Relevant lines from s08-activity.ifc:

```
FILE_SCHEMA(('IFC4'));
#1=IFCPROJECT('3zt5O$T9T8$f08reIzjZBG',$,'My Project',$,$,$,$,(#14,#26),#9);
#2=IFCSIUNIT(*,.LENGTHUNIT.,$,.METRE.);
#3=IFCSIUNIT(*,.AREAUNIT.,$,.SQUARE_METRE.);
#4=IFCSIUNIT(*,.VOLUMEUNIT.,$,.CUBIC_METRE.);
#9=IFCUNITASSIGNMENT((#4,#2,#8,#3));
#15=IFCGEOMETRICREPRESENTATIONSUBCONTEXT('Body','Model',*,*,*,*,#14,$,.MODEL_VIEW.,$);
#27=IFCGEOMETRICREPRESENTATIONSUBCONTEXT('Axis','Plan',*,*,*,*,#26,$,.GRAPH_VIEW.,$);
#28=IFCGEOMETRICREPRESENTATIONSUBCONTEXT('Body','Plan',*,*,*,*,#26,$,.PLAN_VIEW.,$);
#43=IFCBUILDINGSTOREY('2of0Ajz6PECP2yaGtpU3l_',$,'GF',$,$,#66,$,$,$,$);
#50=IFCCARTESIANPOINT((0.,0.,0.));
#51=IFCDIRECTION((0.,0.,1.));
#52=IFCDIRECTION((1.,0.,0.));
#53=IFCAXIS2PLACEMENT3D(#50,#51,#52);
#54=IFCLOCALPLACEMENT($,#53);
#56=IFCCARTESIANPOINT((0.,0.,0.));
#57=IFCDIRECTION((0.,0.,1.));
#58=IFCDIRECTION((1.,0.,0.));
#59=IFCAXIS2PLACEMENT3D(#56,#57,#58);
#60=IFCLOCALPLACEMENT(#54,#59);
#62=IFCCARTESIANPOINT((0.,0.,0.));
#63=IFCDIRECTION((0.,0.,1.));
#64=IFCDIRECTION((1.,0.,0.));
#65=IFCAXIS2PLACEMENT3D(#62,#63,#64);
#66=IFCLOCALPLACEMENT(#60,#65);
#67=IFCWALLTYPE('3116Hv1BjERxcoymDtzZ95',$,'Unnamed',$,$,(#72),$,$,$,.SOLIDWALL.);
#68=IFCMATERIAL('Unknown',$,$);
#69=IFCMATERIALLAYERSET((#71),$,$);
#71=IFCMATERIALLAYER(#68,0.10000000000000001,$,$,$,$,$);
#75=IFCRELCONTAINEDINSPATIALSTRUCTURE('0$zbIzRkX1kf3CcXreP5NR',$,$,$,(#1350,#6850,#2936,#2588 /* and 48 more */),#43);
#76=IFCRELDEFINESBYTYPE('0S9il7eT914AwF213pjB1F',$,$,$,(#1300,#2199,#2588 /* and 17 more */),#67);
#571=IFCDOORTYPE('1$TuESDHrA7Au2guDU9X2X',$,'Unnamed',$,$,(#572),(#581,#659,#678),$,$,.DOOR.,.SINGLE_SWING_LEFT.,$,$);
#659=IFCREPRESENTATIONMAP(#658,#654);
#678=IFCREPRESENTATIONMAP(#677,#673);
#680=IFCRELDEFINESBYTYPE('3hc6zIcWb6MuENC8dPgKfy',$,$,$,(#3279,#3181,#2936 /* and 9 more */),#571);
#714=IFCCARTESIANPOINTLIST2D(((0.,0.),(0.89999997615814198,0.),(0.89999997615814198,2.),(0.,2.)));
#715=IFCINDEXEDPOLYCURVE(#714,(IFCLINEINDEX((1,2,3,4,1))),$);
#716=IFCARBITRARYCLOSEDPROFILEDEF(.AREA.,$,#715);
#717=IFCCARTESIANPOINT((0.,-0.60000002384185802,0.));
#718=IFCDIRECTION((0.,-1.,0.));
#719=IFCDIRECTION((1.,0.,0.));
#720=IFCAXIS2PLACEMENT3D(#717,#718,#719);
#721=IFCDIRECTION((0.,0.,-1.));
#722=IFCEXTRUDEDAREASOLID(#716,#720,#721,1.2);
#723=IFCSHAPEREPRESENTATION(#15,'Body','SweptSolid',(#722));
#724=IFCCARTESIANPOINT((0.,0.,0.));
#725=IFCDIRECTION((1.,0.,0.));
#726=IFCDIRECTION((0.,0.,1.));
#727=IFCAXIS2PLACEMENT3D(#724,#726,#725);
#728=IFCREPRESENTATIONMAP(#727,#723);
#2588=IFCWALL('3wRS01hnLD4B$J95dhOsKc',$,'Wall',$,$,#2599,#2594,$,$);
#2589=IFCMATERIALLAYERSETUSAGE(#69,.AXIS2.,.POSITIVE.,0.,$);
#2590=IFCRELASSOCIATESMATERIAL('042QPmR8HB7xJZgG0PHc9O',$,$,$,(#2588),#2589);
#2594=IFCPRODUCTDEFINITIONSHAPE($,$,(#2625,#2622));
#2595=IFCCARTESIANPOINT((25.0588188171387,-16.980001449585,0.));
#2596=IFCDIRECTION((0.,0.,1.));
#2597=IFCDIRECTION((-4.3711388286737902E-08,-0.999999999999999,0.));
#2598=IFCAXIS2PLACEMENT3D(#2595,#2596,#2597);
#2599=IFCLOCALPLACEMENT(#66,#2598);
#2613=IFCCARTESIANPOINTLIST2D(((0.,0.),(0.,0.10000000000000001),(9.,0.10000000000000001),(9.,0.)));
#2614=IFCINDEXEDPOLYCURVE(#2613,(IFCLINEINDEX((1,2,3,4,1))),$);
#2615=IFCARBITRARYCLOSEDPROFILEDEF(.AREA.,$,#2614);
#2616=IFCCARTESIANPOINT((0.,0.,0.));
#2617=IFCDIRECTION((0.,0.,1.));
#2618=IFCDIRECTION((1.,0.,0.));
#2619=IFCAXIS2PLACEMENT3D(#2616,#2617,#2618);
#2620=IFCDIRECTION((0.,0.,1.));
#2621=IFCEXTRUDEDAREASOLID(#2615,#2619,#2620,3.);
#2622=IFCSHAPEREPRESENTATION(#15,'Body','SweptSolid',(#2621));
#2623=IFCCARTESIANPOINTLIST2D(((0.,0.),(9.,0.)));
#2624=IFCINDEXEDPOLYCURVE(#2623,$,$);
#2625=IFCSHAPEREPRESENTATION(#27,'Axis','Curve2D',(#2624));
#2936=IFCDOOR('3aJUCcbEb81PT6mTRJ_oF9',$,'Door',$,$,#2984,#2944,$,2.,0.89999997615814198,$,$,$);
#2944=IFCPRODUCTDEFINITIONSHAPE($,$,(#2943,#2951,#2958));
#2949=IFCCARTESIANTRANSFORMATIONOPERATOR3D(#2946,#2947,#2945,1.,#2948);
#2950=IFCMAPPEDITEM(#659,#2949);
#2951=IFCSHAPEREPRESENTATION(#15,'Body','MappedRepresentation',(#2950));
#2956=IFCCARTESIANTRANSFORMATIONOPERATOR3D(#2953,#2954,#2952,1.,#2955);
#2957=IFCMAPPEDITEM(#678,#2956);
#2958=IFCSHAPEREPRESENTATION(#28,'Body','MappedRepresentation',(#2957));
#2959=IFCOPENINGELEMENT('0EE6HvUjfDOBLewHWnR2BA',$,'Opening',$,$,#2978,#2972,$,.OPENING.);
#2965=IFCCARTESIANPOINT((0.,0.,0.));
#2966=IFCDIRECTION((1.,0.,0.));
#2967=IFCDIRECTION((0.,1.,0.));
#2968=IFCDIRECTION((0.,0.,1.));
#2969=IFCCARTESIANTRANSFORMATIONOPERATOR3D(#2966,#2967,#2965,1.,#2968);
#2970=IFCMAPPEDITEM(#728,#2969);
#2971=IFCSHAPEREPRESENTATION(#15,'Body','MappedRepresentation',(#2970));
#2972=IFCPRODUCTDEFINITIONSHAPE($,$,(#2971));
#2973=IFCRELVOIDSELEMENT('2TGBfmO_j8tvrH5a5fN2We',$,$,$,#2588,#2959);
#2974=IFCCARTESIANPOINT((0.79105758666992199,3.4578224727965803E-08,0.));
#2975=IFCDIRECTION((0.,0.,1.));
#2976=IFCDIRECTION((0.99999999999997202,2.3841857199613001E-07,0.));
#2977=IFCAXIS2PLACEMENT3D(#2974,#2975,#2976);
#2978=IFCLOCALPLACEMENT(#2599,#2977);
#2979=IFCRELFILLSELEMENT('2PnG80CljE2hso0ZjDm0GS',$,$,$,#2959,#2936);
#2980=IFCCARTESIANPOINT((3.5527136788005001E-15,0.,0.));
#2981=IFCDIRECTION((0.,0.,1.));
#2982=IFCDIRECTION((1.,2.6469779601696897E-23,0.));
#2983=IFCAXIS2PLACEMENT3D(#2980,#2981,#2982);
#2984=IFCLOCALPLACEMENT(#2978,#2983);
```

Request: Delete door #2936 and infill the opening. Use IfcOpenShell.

```python
import ifcopenshell
import ifcopenshell.api.feature
import ifcopenshell.api.root
import ifcopenshell.geom
import ifcopenshell.util.shape

model = ifcopenshell.open("s08-activity.ifc")
settings = ifcopenshell.geom.settings()


def volume(element):
    """Net volume in cubic metres, openings subtracted."""
    shape = ifcopenshell.geom.create_shape(settings, element)
    return ifcopenshell.util.shape.get_volume(shape.geometry)


door = model.by_guid("3aJUCcbEb81PT6mTRJ_oF9")
opening = door.FillsVoids[0].RelatingOpeningElement
wall = opening.VoidsElements[0].RelatingBuildingElement
before = volume(wall)

ifcopenshell.api.root.remove_product(model, product=door)
ifcopenshell.api.feature.remove_feature(model, feature=opening)

after = volume(wall)

print(f"wall volume {before:.3f} -> {after:.3f} m3")

model.write("s08-activity_rev.ifc")
```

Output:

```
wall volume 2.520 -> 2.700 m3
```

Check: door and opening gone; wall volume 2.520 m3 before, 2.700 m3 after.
